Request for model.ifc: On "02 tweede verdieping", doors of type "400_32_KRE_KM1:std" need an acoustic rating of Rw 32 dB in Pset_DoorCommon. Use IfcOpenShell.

First a look at what the model holds.

```python
import ifcopenshell
import ifcopenshell.util.element

model = ifcopenshell.open("model.ifc")
print(model.schema)
storey = next(s for s in model.by_type("IfcBuildingStorey") if s.Name == "02 tweede verdieping")
doors = [e for e in ifcopenshell.util.element.get_decomposition(storey) if e.is_a("IfcDoor")]
seen = {}
for e in doors:
    element_type = ifcopenshell.util.element.get_type(e)
    key = (element_type.Name if element_type != e and element_type else None, ifcopenshell.util.element.get_pset(e, "Pset_DoorCommon", "AcousticRating"))
    seen[key] = seen.get(key, 0) + 1
for (name, value), count in sorted(seen.items(), key=str):
    print(count, "x", name, "|", value)
```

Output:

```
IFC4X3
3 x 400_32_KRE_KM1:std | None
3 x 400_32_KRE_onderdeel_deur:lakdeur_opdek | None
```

```python
import ifcopenshell
import ifcopenshell.api.pset
import ifcopenshell.util.element

model = ifcopenshell.open("model.ifc")

storey = next(s for s in model.by_type("IfcBuildingStorey") if s.Name == "02 tweede verdieping")
doors = [e for e in ifcopenshell.util.element.get_decomposition(storey) if e.is_a("IfcDoor")]

count = 0
for e in doors:
    element_type = ifcopenshell.util.element.get_type(e)
    if element_type in (None, e) or element_type.Name != "400_32_KRE_KM1:std":
        continue
    # add_pset returns the element's existing set when there is one.
    pset = ifcopenshell.api.pset.add_pset(model, product=e, name="Pset_DoorCommon")
    ifcopenshell.api.pset.edit_pset(model, pset=pset, properties={"AcousticRating": "Rw 32 dB"})
    count += 1

print(count, "doors updated")

model.write("model_rev.ifc")
```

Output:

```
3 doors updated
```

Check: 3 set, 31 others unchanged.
